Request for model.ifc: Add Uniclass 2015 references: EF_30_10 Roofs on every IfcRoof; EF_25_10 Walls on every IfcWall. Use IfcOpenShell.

First a look at what the model holds.

```python
import ifcopenshell

model = ifcopenshell.open("model.ifc")
print(model.schema)
print("classifications:", [c.Name for c in model.by_type("IfcClassification")])
for ifc_class in ("IfcDoor", "IfcRoof", "IfcStair", "IfcWall", "IfcWindow"):
    print(ifc_class, len(model.by_type(ifc_class)))
```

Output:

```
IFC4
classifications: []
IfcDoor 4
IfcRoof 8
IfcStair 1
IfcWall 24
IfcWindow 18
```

```python
import ifcopenshell
import ifcopenshell.api.classification

model = ifcopenshell.open("model.ifc")

system = ifcopenshell.api.classification.add_classification(model, classification="Uniclass 2015")

codes = {
    "IfcRoof": ("EF_30_10", "Roofs"),
    "IfcWall": ("EF_25_10", "Walls"),
}
for ifc_class, (code, name) in codes.items():
    products = model.by_type(ifc_class)
    ifcopenshell.api.classification.add_reference(
        model, products=products, classification=system, identification=code, name=name
    )
    print(code, len(products))

model.write("model_edited.ifc")
```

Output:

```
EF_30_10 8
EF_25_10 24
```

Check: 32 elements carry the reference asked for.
